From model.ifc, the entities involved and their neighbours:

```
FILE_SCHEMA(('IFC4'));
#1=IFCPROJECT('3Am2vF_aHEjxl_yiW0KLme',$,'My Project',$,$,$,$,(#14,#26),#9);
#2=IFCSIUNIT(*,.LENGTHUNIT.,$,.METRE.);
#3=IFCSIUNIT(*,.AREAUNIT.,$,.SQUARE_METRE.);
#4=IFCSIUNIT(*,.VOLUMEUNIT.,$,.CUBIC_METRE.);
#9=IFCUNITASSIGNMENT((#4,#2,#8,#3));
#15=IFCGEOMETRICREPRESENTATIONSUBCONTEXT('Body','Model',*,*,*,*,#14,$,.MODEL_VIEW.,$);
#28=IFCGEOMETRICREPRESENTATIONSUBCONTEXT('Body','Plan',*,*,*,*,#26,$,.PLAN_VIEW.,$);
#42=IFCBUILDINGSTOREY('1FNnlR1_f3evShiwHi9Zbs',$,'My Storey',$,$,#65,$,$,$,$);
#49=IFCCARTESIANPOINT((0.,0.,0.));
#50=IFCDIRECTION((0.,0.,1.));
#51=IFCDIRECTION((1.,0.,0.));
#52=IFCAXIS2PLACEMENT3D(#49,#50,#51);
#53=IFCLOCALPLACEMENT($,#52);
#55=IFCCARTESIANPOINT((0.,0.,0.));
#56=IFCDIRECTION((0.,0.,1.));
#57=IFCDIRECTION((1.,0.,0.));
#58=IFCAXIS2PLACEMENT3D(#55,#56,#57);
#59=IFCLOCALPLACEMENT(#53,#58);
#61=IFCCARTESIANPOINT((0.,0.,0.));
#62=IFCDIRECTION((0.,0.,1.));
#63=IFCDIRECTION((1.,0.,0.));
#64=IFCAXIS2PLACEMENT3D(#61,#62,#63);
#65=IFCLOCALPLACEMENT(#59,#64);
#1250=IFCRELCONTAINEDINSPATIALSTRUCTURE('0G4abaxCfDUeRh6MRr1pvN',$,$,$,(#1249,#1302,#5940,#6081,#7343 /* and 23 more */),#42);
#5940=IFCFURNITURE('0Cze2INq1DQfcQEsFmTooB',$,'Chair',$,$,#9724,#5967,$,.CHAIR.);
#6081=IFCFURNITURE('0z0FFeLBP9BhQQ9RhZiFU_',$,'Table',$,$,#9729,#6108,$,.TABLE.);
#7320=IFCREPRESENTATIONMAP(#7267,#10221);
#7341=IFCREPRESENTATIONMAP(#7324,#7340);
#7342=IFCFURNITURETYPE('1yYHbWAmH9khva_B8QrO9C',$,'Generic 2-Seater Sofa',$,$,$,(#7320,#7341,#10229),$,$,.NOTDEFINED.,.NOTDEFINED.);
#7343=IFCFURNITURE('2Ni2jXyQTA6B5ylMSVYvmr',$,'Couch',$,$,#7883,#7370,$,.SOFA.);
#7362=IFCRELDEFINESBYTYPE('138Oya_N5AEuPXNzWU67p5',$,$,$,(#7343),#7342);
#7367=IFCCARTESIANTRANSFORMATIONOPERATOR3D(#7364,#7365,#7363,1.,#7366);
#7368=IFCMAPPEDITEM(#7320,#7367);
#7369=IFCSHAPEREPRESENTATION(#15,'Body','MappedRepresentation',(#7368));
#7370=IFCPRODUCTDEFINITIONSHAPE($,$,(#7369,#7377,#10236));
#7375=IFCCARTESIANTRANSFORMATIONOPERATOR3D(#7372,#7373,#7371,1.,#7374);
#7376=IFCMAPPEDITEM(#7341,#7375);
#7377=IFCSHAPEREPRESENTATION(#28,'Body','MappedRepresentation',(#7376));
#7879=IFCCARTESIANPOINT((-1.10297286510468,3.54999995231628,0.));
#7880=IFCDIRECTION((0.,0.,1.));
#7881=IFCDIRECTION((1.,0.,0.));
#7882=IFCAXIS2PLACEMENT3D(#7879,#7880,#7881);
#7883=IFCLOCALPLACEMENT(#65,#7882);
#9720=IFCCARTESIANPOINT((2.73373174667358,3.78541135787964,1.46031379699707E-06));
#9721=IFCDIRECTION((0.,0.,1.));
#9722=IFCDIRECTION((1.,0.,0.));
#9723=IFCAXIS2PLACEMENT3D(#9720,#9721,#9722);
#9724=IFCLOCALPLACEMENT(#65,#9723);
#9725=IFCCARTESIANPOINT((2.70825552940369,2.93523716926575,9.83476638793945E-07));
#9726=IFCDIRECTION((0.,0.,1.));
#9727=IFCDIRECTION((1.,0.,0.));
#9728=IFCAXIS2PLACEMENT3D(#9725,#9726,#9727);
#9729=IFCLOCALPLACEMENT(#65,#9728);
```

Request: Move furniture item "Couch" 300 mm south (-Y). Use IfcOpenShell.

```python
import ifcopenshell
import ifcopenshell.api.geometry
import ifcopenshell.util.placement
import ifcopenshell.util.unit

model = ifcopenshell.open("model.ifc")
unit_scale = ifcopenshell.util.unit.calculate_unit_scale(model)

item = model.by_guid("2Ni2jXyQTA6B5ylMSVYvmr")
matrix = ifcopenshell.util.placement.get_local_placement(item.ObjectPlacement)
matrix[1, 3] -= 0.3 / unit_scale
ifcopenshell.api.geometry.edit_object_placement(model, product=item, matrix=matrix, is_si=False)

print(ifcopenshell.util.placement.get_local_placement(item.ObjectPlacement).round(3) + 0.0)

model.write("model_edited.ifc")
```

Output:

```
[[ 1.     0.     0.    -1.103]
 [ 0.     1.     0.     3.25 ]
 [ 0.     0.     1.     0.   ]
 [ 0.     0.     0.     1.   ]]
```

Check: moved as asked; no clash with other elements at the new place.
